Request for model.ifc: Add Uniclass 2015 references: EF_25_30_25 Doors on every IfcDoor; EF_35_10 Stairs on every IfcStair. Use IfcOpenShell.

First a look at what the model holds.

```python
import ifcopenshell

model = ifcopenshell.open("model.ifc")
print(model.schema)
print("classifications:", [c.Name for c in model.by_type("IfcClassification")])
for ifc_class in ("IfcDoor", "IfcRoof", "IfcStair", "IfcWall", "IfcWindow"):
    print(ifc_class, len(model.by_type(ifc_class)))
```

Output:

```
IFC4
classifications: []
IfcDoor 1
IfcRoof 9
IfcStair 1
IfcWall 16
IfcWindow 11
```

```python
import ifcopenshell
import ifcopenshell.api.classification

model = ifcopenshell.open("model.ifc")

system = ifcopenshell.api.classification.add_classification(model, classification="Uniclass 2015")

codes = {
    "IfcDoor": ("EF_25_30_25", "Doors"),
    "IfcStair": ("EF_35_10", "Stairs"),
}
for ifc_class, (code, name) in codes.items():
    products = model.by_type(ifc_class)
    ifcopenshell.api.classification.add_reference(
        model, products=products, classification=system, identification=code, name=name
    )
    print(code, len(products))

model.write("model_edited.ifc")
```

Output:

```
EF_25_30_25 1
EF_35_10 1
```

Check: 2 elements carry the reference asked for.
